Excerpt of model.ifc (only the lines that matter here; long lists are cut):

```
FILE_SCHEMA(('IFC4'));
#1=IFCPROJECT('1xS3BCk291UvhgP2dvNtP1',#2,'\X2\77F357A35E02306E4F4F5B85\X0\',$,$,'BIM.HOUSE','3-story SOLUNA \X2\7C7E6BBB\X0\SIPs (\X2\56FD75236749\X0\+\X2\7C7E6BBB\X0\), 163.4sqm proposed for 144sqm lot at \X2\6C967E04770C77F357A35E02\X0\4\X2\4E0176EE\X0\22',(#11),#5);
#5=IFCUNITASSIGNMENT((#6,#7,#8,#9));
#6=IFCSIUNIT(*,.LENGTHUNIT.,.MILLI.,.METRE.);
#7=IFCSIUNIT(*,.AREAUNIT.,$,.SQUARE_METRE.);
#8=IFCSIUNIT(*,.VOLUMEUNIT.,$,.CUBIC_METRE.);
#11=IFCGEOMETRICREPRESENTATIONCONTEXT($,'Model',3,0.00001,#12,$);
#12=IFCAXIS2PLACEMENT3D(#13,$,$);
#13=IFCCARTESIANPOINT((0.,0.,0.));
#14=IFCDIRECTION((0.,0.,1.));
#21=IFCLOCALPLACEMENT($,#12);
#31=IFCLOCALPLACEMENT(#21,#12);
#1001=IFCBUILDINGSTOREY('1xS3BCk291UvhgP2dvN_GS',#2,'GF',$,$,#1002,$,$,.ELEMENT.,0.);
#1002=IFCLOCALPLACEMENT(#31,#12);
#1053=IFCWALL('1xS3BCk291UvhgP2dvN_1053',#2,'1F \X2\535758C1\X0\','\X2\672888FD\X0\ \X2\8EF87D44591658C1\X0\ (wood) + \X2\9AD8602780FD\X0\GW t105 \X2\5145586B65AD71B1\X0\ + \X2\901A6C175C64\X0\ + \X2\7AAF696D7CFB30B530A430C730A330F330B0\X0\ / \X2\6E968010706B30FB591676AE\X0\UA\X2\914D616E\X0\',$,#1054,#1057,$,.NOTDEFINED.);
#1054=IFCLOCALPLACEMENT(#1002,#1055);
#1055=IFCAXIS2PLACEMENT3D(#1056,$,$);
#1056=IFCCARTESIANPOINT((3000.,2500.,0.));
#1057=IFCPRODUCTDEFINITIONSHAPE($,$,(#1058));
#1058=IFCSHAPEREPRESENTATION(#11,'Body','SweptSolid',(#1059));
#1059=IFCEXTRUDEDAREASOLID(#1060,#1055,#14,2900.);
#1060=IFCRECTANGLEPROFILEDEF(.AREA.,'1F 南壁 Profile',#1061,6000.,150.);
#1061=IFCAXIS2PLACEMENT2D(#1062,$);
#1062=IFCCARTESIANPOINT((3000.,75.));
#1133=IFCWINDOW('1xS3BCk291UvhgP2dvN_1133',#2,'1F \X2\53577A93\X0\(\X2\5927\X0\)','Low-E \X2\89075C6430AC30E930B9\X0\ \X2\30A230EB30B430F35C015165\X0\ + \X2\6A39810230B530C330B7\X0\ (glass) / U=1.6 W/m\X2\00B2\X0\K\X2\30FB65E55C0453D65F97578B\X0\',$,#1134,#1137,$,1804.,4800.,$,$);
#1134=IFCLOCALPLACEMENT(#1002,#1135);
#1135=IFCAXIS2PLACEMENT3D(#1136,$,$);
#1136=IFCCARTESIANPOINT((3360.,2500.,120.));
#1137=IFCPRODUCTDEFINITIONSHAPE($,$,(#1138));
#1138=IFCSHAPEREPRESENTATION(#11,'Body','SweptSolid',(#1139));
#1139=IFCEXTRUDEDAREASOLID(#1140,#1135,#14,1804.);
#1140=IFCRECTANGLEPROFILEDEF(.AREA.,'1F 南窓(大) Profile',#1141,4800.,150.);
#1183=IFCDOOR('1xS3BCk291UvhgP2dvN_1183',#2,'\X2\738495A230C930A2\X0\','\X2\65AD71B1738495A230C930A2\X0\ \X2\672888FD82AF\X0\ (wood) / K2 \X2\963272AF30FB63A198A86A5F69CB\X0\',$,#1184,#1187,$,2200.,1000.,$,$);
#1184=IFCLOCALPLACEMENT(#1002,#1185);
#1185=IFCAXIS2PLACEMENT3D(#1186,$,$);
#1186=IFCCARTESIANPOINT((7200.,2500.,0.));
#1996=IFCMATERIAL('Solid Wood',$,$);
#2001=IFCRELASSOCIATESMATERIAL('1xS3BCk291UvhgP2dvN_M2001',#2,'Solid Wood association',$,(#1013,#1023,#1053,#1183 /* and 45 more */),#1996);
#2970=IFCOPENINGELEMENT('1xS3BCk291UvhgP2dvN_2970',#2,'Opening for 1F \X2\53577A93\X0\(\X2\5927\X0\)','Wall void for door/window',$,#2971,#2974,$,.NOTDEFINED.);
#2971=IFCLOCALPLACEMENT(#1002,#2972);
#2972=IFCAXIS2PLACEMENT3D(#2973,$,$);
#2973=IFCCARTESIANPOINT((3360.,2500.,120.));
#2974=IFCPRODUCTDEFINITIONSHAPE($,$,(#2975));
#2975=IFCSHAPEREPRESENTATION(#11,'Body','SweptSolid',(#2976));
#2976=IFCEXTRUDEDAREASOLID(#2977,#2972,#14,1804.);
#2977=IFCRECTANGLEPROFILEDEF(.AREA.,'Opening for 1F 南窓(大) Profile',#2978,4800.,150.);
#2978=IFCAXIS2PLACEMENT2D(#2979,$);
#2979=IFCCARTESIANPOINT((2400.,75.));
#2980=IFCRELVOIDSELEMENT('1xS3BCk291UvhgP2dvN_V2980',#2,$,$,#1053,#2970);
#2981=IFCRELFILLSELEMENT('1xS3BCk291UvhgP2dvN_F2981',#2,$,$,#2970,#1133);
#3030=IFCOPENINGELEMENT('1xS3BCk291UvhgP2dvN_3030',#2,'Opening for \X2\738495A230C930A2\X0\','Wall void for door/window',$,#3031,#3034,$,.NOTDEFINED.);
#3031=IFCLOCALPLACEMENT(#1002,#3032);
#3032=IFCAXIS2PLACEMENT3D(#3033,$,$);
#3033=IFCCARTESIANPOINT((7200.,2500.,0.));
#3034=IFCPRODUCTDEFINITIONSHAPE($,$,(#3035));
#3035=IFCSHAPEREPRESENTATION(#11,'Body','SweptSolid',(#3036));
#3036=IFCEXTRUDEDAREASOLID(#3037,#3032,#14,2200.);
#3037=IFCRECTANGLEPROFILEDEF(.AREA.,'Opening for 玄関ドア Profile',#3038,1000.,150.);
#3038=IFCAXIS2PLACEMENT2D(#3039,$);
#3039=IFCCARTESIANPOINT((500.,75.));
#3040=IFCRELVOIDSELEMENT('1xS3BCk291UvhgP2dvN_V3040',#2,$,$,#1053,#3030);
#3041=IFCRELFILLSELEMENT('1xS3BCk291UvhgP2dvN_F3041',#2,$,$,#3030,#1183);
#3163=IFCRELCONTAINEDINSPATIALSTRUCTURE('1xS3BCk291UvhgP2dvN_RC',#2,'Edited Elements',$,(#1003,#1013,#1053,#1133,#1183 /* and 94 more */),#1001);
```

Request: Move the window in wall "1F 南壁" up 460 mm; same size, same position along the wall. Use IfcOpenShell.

```python
import numpy as np
import ifcopenshell
import ifcopenshell.api.geometry
import ifcopenshell.util.placement
import ifcopenshell.util.unit

model = ifcopenshell.open("model.ifc")
unit_scale = ifcopenshell.util.unit.calculate_unit_scale(model)

window = model.by_guid("1xS3BCk291UvhgP2dvN_1133")
opening = window.FillsVoids[0].RelatingOpeningElement
dz = 460.0

shift = np.array([0.0, 0.0, dz])
# The window is not placed relative to its opening, so move both.
for product in (opening, window):
    matrix = ifcopenshell.util.placement.get_local_placement(product.ObjectPlacement)
    matrix[:3, 3] += shift
    ifcopenshell.api.geometry.edit_object_placement(model, product=product, matrix=matrix, is_si=False)

print(f"moved by {dz * unit_scale:+.3f} m")

model.write("model_rev.ifc")
```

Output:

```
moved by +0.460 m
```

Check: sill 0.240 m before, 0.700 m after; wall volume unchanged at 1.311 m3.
